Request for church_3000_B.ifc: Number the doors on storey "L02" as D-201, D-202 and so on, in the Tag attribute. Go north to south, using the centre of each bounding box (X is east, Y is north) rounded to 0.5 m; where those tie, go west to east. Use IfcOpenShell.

First a look at what the model holds.

```python
import ifcopenshell
import ifcopenshell.util.element
import ifcopenshell.util.placement

model = ifcopenshell.open("church_3000_B.ifc")
print(model.schema)
storey = next(s for s in model.by_type("IfcBuildingStorey") if s.Name == "L02")
doors = [e for e in ifcopenshell.util.element.get_decomposition(storey) if e.is_a("IfcDoor")]
for e in sorted(doors, key=lambda e: e.id()):
    origin = ifcopenshell.util.placement.get_local_placement(e.ObjectPlacement)[:3, 3]
    print(e.id(), e.Tag, e.Name, origin.round(2) + 0.0, sep=" | ")
```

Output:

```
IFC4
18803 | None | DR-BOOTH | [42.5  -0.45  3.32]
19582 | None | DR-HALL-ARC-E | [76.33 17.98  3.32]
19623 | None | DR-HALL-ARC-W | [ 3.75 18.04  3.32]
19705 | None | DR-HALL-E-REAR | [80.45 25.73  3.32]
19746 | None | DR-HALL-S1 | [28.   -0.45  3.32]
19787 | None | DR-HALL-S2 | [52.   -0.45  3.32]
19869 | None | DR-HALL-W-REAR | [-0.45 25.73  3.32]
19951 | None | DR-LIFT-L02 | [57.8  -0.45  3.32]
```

```python
import ifcopenshell
import ifcopenshell.geom
import ifcopenshell.util.element
import ifcopenshell.util.shape

model = ifcopenshell.open("church_3000_B.ifc")
settings = ifcopenshell.geom.settings()
settings.set("use-world-coords", True)


def centre(element):
    shape = ifcopenshell.geom.create_shape(settings, element)
    return ifcopenshell.util.shape.get_bbox_centroid(shape.geometry)


storey = next(s for s in model.by_type("IfcBuildingStorey") if s.Name == "L02")
doors = [e for e in ifcopenshell.util.element.get_decomposition(storey) if e.is_a("IfcDoor")]

# Insertion points can sit at a corner or the storey origin, so sort by the geometry (in metres).
centres = {e: centre(e) for e in doors}
doors.sort(key=lambda e: (-round(centres[e][1] / 0.5), centres[e][0]))

for i, e in enumerate(doors, start=1):
    number = f"D-2{i:02d}"
    e.Tag = number
    print(e.id(), number)

model.write("church_3000_B_v2.ifc")
```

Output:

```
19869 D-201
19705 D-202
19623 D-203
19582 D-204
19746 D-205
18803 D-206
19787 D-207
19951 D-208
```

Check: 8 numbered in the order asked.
